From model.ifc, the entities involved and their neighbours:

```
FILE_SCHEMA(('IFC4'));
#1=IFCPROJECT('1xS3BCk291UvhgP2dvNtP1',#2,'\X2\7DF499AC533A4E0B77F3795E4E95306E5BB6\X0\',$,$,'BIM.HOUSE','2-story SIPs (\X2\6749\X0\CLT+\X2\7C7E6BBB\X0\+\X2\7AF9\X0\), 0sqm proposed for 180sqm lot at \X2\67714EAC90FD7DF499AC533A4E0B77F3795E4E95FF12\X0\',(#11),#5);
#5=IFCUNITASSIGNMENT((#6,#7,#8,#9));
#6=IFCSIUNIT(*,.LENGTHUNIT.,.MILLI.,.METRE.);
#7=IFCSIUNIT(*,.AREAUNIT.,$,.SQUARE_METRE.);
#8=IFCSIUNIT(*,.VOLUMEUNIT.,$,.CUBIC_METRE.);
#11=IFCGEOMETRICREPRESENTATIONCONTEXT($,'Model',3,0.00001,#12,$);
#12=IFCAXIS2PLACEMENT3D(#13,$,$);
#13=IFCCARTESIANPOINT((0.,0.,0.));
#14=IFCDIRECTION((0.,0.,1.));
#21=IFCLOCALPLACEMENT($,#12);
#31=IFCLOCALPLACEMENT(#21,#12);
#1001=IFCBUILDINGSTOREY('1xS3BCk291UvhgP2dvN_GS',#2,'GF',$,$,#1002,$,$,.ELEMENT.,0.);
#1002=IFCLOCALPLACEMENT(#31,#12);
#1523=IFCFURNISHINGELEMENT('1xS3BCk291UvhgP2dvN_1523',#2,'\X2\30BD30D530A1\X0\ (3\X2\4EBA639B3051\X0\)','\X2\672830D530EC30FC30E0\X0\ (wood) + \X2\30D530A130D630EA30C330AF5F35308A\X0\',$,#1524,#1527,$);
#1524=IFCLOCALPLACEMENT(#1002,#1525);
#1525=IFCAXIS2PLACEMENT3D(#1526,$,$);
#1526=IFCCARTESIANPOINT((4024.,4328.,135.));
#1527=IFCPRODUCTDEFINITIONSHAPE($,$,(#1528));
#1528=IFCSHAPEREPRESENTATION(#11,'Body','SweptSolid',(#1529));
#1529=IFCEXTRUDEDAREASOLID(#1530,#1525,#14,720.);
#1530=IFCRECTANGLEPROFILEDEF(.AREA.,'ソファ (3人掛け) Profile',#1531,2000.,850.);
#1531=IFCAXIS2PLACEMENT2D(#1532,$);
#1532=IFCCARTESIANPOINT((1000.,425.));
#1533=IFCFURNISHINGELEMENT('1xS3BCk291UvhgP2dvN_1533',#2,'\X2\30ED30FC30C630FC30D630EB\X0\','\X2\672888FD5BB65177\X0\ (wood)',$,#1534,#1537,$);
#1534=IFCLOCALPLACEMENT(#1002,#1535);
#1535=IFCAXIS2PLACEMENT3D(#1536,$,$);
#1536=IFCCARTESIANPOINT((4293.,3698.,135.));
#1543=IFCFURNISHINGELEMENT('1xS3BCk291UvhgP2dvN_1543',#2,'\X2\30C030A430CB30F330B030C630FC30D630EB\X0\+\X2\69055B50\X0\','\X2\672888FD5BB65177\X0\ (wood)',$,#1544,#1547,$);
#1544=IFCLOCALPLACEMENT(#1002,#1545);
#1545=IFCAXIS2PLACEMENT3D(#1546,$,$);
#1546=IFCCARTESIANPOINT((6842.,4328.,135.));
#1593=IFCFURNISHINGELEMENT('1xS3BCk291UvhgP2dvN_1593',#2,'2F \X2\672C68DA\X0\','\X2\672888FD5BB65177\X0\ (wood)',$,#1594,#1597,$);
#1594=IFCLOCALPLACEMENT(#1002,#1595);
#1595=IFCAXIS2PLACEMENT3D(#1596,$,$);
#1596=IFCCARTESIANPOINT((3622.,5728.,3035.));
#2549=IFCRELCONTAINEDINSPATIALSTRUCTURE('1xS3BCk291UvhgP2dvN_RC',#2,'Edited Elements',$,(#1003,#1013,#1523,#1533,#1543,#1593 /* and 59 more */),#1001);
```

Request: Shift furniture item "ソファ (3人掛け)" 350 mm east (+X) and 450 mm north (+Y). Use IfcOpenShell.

```python
import ifcopenshell
import ifcopenshell.api.geometry
import ifcopenshell.util.placement
import ifcopenshell.util.unit

model = ifcopenshell.open("model.ifc")
unit_scale = ifcopenshell.util.unit.calculate_unit_scale(model)

item = model.by_guid("1xS3BCk291UvhgP2dvN_1523")
matrix = ifcopenshell.util.placement.get_local_placement(item.ObjectPlacement)
matrix[0, 3] += 0.35 / unit_scale
matrix[1, 3] += 0.45 / unit_scale
ifcopenshell.api.geometry.edit_object_placement(model, product=item, matrix=matrix, is_si=False)

print(ifcopenshell.util.placement.get_local_placement(item.ObjectPlacement).round(3) + 0.0)

model.write("model-out.ifc")
```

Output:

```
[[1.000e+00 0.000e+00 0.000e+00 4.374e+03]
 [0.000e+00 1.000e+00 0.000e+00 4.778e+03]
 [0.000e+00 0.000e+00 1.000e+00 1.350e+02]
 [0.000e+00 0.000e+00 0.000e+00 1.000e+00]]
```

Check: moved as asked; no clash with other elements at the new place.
